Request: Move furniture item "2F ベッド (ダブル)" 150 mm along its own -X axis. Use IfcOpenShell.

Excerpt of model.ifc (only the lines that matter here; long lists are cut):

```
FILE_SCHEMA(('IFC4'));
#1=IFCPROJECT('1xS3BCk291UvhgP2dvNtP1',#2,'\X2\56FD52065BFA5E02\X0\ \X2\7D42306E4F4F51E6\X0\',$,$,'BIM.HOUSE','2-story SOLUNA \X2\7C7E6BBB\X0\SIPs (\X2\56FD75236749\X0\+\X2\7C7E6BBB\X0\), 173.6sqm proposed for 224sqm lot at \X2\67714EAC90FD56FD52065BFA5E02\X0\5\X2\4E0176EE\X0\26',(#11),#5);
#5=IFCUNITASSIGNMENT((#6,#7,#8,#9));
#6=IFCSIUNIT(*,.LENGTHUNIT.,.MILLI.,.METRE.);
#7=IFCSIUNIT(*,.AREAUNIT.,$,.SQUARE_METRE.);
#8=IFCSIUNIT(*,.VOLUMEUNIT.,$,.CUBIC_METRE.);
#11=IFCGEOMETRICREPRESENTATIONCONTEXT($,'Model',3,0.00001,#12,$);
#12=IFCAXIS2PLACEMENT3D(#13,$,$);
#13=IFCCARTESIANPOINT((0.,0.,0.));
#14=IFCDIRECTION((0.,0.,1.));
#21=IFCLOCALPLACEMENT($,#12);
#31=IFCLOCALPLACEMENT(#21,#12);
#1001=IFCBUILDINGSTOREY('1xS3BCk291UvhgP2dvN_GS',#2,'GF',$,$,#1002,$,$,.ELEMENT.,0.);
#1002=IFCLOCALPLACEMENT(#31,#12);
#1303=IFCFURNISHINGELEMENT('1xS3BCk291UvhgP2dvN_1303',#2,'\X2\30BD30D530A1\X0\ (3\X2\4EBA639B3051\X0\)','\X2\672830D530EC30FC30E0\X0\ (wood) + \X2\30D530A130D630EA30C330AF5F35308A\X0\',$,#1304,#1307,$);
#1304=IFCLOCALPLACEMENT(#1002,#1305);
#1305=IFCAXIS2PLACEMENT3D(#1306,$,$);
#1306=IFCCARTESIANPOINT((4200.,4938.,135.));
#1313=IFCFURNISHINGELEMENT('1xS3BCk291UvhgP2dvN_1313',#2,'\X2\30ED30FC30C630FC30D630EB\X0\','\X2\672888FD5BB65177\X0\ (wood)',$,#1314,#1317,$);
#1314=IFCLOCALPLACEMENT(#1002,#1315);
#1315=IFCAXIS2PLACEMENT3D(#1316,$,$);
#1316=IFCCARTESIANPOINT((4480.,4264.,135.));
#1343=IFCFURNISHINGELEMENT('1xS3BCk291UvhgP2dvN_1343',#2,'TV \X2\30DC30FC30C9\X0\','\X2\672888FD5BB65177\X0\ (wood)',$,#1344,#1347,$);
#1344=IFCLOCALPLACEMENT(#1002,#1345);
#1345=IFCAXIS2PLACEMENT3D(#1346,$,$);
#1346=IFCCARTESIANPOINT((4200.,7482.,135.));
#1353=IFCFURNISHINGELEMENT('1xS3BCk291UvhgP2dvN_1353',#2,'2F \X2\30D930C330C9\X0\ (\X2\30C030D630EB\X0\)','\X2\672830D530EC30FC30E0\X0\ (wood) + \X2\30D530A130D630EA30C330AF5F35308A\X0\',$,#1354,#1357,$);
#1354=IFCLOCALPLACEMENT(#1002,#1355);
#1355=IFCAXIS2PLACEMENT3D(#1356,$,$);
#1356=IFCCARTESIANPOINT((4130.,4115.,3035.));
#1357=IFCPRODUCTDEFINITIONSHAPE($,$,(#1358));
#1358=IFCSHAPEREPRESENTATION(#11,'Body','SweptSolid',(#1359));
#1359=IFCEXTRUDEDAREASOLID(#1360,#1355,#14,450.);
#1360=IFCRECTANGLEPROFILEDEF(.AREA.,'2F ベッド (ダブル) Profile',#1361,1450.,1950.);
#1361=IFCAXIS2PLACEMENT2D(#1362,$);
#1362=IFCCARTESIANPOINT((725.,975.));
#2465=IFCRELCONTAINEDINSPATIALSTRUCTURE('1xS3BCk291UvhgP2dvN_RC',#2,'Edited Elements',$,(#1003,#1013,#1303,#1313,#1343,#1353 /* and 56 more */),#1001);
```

```python
import ifcopenshell
import ifcopenshell.api.geometry
import ifcopenshell.util.placement
import ifcopenshell.util.unit

model = ifcopenshell.open("model.ifc")
unit_scale = ifcopenshell.util.unit.calculate_unit_scale(model)

item = model.by_id(1353)
matrix = ifcopenshell.util.placement.get_local_placement(item.ObjectPlacement)
matrix[:3, 3] -= matrix[:3, 0] * 0.15 / unit_scale
ifcopenshell.api.geometry.edit_object_placement(model, product=item, matrix=matrix, is_si=False)

print(ifcopenshell.util.placement.get_local_placement(item.ObjectPlacement).round(3) + 0.0)

model.write("model_updated.ifc")
```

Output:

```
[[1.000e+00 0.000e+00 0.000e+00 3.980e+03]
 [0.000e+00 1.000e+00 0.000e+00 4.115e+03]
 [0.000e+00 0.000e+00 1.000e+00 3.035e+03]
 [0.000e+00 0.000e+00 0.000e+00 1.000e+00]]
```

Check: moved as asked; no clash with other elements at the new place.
